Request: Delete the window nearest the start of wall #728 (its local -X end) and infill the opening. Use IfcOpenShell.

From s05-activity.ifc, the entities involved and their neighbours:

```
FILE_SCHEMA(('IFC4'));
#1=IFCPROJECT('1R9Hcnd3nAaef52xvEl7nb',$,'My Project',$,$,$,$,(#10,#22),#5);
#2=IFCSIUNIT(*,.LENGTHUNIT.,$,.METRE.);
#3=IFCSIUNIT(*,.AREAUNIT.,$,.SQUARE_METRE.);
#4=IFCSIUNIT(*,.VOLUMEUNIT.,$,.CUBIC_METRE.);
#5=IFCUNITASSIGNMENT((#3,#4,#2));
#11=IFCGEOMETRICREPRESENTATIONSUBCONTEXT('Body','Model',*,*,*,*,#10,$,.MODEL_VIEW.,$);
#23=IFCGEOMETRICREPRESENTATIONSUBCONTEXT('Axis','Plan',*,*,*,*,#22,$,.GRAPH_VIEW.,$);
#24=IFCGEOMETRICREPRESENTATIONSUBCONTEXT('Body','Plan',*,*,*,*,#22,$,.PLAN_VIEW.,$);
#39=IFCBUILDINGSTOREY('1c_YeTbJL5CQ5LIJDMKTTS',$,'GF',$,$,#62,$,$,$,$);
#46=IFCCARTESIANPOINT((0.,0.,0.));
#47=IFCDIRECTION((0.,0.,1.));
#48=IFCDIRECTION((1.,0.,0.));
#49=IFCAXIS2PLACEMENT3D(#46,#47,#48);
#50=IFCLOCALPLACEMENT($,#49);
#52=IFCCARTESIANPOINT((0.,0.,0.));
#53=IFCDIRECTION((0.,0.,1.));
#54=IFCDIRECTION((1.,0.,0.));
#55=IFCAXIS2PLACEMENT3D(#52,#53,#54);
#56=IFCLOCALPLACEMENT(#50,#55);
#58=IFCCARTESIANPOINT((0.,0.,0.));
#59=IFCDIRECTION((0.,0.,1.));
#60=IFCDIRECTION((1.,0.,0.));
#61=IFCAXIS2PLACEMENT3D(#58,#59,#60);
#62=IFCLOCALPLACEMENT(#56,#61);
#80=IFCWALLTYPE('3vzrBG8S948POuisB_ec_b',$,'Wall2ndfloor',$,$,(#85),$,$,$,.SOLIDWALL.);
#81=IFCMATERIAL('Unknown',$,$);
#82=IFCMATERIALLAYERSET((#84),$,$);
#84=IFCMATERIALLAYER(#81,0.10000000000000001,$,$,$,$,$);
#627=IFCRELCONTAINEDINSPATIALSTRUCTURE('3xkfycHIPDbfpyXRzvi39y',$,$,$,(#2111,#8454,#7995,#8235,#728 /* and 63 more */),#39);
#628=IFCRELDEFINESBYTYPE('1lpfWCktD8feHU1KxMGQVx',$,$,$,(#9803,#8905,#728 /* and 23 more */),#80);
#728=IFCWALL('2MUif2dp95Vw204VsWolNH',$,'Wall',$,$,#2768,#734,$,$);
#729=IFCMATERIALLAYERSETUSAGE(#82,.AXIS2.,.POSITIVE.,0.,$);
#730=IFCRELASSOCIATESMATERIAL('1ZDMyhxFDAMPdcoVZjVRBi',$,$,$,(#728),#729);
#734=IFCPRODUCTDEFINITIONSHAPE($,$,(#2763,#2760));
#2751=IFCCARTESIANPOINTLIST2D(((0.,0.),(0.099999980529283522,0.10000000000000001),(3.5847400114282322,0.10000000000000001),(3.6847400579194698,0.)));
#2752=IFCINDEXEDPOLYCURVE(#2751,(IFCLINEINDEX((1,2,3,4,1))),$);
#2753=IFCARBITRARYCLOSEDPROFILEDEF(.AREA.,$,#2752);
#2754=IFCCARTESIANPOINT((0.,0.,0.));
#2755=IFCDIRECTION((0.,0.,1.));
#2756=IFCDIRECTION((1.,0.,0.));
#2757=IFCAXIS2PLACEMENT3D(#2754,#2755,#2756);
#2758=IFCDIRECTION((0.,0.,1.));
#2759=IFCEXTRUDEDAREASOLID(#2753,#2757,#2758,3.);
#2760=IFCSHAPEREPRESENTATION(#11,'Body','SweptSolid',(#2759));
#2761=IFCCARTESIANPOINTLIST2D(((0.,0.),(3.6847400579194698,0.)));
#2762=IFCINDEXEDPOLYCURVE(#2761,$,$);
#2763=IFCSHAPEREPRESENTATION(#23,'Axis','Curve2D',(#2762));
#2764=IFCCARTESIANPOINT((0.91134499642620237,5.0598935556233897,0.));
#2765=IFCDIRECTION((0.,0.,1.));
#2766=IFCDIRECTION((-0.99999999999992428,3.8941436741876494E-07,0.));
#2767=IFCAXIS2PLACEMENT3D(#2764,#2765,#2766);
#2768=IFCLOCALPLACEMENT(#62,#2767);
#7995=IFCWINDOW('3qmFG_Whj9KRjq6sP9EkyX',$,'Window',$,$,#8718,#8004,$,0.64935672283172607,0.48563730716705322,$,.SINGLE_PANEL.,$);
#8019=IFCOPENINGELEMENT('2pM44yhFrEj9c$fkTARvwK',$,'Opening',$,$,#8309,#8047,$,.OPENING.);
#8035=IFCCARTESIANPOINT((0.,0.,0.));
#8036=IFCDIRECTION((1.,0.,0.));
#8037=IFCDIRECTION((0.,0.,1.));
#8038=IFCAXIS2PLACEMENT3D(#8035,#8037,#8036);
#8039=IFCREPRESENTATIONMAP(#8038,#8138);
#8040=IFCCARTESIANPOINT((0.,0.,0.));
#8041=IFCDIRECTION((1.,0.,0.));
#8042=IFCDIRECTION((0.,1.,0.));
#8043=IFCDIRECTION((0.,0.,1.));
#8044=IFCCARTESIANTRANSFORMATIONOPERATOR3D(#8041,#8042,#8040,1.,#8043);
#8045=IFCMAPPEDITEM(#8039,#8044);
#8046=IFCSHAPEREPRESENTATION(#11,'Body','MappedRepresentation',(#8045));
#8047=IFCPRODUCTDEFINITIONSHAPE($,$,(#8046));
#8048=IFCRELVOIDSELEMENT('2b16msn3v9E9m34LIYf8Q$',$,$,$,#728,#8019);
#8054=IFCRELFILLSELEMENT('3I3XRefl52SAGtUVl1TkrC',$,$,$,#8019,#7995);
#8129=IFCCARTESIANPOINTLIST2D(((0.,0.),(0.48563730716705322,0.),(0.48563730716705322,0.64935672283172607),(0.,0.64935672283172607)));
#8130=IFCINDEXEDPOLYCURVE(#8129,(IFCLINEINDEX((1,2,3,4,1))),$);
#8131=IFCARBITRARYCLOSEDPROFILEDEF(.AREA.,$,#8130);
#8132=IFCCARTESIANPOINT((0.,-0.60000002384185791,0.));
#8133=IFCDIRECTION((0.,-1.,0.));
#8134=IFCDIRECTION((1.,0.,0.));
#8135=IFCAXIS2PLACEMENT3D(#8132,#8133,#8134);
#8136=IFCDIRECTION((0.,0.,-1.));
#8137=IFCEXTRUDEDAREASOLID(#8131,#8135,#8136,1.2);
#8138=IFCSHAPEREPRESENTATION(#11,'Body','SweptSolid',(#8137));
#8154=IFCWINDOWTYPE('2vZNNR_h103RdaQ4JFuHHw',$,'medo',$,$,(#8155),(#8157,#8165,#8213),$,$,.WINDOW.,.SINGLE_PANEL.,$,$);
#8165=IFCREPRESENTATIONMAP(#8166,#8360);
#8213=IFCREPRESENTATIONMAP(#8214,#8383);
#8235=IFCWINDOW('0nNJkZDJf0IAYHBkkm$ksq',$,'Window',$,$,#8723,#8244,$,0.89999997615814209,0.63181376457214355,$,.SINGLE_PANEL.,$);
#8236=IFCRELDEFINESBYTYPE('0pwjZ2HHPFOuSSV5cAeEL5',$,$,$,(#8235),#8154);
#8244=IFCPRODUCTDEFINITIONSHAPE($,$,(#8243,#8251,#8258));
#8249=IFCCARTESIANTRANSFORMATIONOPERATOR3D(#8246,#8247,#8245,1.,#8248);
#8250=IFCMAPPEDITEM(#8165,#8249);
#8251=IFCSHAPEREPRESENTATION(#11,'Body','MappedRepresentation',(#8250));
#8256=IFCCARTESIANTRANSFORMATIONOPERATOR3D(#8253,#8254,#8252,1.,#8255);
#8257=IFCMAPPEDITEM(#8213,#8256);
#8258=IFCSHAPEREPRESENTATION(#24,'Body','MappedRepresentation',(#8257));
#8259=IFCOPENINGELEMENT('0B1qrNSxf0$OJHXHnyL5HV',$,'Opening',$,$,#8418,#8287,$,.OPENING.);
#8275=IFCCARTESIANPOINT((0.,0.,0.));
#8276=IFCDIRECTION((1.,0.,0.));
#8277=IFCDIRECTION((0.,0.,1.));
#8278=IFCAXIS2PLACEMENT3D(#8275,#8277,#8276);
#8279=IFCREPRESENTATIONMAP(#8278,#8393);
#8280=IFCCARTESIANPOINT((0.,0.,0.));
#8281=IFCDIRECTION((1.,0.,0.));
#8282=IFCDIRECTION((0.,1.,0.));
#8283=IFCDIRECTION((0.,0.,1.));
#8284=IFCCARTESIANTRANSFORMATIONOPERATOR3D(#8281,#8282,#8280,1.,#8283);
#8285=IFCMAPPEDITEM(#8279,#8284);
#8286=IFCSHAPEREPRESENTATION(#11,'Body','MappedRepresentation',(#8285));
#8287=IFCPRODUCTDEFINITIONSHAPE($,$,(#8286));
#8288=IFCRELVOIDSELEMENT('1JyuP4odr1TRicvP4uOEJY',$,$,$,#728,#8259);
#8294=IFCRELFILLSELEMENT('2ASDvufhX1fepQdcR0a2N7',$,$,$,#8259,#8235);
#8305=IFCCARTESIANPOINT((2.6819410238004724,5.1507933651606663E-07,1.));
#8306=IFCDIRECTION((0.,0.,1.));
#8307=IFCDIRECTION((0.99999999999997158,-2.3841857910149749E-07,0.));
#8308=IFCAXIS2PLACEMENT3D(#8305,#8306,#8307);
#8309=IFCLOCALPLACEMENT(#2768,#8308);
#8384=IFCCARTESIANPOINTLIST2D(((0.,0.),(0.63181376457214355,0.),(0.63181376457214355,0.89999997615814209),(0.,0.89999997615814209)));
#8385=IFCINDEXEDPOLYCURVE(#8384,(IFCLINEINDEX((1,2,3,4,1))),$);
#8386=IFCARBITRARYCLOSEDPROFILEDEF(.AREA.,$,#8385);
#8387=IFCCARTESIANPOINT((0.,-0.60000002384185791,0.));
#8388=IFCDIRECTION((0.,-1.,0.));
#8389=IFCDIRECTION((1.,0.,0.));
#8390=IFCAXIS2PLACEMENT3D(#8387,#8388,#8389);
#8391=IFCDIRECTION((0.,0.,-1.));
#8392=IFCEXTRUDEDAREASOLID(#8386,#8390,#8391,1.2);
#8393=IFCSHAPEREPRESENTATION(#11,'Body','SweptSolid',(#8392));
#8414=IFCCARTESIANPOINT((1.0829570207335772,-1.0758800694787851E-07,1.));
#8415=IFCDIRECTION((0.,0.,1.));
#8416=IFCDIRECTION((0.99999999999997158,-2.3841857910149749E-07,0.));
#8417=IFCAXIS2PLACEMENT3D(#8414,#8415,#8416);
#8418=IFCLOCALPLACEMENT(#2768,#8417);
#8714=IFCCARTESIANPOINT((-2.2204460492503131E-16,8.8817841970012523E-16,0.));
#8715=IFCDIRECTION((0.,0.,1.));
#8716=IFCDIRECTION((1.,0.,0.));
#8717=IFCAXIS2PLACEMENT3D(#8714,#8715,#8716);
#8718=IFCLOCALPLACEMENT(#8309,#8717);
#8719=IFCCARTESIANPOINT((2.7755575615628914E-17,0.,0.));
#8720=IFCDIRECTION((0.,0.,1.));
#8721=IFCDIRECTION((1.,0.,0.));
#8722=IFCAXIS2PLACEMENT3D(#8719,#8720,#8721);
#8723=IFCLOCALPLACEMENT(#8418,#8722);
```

```python
import ifcopenshell
import ifcopenshell.api.feature
import ifcopenshell.api.root
import ifcopenshell.geom
import ifcopenshell.util.shape

model = ifcopenshell.open("s05-activity.ifc")
settings = ifcopenshell.geom.settings()


def volume(element):
    """Net volume in cubic metres, openings subtracted."""
    shape = ifcopenshell.geom.create_shape(settings, element)
    return ifcopenshell.util.shape.get_volume(shape.geometry)


window = model.by_id(8235)
opening = window.FillsVoids[0].RelatingOpeningElement
wall = opening.VoidsElements[0].RelatingBuildingElement
before = volume(wall)

ifcopenshell.api.root.remove_product(model, product=window)
ifcopenshell.api.feature.remove_feature(model, feature=opening)

after = volume(wall)

print(f"wall volume {before:.3f} -> {after:.3f} m3")

model.write("s05-activity-out.ifc")
```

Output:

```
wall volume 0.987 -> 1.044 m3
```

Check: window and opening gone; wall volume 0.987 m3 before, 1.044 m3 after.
